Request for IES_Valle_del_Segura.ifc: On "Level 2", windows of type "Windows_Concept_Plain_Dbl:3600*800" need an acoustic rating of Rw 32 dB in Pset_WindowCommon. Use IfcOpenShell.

First a look at what the model holds.

```python
import ifcopenshell
import ifcopenshell.util.element

model = ifcopenshell.open("IES_Valle_del_Segura.ifc")
print(model.schema)
storey = next(s for s in model.by_type("IfcBuildingStorey") if s.Name == "Level 2")
windows = [e for e in ifcopenshell.util.element.get_decomposition(storey) if e.is_a("IfcWindow")]
seen = {}
for e in windows:
    element_type = ifcopenshell.util.element.get_type(e)
    key = (element_type.Name if element_type != e and element_type else None, ifcopenshell.util.element.get_pset(e, "Pset_WindowCommon", "AcousticRating"))
    seen[key] = seen.get(key, 0) + 1
for (name, value), count in sorted(seen.items(), key=str):
    print(count, "x", name, "|", value)
```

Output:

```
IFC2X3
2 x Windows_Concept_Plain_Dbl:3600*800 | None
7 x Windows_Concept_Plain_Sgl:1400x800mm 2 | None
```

```python
import ifcopenshell
import ifcopenshell.api.pset
import ifcopenshell.util.element

model = ifcopenshell.open("IES_Valle_del_Segura.ifc")

storey = next(s for s in model.by_type("IfcBuildingStorey") if s.Name == "Level 2")
windows = [e for e in ifcopenshell.util.element.get_decomposition(storey) if e.is_a("IfcWindow")]

count = 0
for e in windows:
    element_type = ifcopenshell.util.element.get_type(e)
    if element_type in (None, e) or element_type.Name != "Windows_Concept_Plain_Dbl:3600*800":
        continue
    # add_pset returns the element's existing set when there is one.
    pset = ifcopenshell.api.pset.add_pset(model, product=e, name="Pset_WindowCommon")
    ifcopenshell.api.pset.edit_pset(model, pset=pset, properties={"AcousticRating": "Rw 32 dB"})
    count += 1

print(count, "windows updated")

model.write("IES_Valle_del_Segura_rev.ifc")
```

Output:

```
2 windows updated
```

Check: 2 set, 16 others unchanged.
